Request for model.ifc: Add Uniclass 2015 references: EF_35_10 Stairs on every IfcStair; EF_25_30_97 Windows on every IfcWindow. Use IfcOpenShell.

First a look at what the model holds.

```python
import ifcopenshell

model = ifcopenshell.open("model.ifc")
print(model.schema)
print("classifications:", [c.Name for c in model.by_type("IfcClassification")])
for ifc_class in ("IfcDoor", "IfcRoof", "IfcStair", "IfcWall", "IfcWindow"):
    print(ifc_class, len(model.by_type(ifc_class)))
```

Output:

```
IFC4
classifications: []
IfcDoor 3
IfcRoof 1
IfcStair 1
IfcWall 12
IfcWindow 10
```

```python
import ifcopenshell
import ifcopenshell.api.classification

model = ifcopenshell.open("model.ifc")

system = ifcopenshell.api.classification.add_classification(model, classification="Uniclass 2015")

codes = {
    "IfcStair": ("EF_35_10", "Stairs"),
    "IfcWindow": ("EF_25_30_97", "Windows"),
}
for ifc_class, (code, name) in codes.items():
    products = model.by_type(ifc_class)
    ifcopenshell.api.classification.add_reference(
        model, products=products, classification=system, identification=code, name=name
    )
    print(code, len(products))

model.write("model-out.ifc")
```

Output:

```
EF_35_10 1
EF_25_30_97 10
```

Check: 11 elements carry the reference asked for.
